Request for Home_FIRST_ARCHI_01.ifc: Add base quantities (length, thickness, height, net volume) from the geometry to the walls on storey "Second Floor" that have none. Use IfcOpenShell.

First a look at what the model holds.

```python
import ifcopenshell
import ifcopenshell.util.element
import ifcopenshell.util.unit

model = ifcopenshell.open("Home_FIRST_ARCHI_01.ifc")
print(model.schema)
for unit_type in ("LENGTHUNIT", "AREAUNIT", "VOLUMEUNIT"):
    print(unit_type, ifcopenshell.util.unit.calculate_unit_scale(model, unit_type))
storey = next(s for s in model.by_type("IfcBuildingStorey") if s.Name == "Second Floor")
walls = [e for e in ifcopenshell.util.element.get_decomposition(storey) if e.is_a("IfcWall")]
for e in sorted(walls, key=lambda e: e.id()):
    print(e.id(), e.is_a(), e.Name, list(ifcopenshell.util.element.get_psets(e, qtos_only=True)), sep=" | ")
```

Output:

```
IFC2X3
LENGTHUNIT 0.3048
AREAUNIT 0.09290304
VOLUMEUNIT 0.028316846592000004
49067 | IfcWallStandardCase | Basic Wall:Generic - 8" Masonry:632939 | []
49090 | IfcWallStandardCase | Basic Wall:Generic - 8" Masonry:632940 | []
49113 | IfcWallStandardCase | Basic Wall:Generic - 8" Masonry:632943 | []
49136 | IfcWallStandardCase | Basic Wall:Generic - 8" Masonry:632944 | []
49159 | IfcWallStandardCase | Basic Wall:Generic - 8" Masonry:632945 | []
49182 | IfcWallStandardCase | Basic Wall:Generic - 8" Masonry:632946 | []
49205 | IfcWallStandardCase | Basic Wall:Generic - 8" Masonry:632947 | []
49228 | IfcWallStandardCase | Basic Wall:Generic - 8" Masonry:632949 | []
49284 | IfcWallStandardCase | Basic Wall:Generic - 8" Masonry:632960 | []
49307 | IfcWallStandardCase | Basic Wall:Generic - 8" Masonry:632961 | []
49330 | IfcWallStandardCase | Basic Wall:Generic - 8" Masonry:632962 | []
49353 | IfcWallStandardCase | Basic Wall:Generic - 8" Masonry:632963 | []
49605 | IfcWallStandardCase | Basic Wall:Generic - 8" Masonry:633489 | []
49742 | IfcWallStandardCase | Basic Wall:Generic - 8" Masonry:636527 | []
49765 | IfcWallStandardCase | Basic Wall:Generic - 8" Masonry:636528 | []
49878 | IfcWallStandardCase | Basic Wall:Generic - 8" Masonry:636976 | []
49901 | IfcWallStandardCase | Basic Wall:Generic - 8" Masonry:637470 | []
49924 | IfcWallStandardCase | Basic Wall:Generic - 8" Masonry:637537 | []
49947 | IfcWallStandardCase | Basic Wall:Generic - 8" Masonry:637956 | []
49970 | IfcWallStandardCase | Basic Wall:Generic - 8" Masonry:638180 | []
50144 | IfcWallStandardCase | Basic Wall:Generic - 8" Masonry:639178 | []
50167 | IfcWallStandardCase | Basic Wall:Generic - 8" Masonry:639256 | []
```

```python
import ifcopenshell
import ifcopenshell.api.pset
import ifcopenshell.geom
import ifcopenshell.util.element
import ifcopenshell.util.shape
import ifcopenshell.util.unit

model = ifcopenshell.open("Home_FIRST_ARCHI_01.ifc")
unit_scale = ifcopenshell.util.unit.calculate_unit_scale(model)
volume_scale = ifcopenshell.util.unit.calculate_unit_scale(model, "VOLUMEUNIT")
settings = ifcopenshell.geom.settings()

storey = next(s for s in model.by_type("IfcBuildingStorey") if s.Name == "Second Floor")
walls = [e for e in ifcopenshell.util.element.get_decomposition(storey) if e.is_a("IfcWall")]

for e in sorted(walls, key=lambda e: e.id()):
    if ifcopenshell.util.element.get_psets(e, qtos_only=True, should_inherit=False):
        continue
    # Geometry comes back in metres, in the element's own axes.
    shape = ifcopenshell.geom.create_shape(settings, e)
    values = {
        "Length": ifcopenshell.util.shape.get_x(shape.geometry) / unit_scale,
        "Width": ifcopenshell.util.shape.get_y(shape.geometry) / unit_scale,
        "Height": ifcopenshell.util.shape.get_z(shape.geometry) / unit_scale,
        "NetVolume": ifcopenshell.util.shape.get_volume(shape.geometry) / volume_scale,
    }
    qto = ifcopenshell.api.pset.add_qto(model, product=e, name="BaseQuantities")
    ifcopenshell.api.pset.edit_qto(model, qto=qto, properties=values)
    print(e.id(), {k: round(v, 3) for k, v in values.items()})

model.write("Home_FIRST_ARCHI_01_rev.ifc")
```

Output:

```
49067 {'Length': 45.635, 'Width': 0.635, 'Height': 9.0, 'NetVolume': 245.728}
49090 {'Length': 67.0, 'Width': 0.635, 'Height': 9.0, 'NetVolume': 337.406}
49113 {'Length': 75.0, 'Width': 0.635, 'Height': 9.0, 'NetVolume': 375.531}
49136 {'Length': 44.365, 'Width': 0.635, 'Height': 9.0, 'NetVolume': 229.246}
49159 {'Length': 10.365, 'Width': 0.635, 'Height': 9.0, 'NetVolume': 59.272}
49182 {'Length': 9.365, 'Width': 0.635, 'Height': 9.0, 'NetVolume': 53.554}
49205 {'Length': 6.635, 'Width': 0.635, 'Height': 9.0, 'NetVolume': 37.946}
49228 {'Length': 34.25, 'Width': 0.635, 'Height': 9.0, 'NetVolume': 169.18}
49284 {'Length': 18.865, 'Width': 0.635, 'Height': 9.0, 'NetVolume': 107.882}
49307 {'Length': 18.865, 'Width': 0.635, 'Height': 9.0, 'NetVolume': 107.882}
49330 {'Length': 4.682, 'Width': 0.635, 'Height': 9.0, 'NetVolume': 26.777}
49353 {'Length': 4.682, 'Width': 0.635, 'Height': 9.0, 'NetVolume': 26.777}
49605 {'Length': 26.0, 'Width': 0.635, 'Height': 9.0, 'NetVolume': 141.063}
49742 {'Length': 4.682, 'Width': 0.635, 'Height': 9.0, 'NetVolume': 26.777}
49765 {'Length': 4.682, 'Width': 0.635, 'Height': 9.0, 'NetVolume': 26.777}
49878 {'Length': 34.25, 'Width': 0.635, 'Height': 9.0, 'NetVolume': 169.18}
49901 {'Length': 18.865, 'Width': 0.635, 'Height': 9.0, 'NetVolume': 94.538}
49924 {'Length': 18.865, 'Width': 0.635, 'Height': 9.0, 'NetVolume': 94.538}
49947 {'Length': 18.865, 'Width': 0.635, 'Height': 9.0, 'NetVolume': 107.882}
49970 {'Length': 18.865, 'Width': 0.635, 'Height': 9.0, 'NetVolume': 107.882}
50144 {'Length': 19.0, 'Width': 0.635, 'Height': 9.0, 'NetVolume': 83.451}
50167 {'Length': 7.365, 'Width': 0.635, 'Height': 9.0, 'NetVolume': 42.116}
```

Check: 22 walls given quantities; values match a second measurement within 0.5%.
